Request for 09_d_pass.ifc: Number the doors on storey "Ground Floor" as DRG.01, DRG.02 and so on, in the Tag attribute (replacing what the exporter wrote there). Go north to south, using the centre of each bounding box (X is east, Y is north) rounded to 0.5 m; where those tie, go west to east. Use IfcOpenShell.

First a look at what the model holds.

```python
import ifcopenshell
import ifcopenshell.util.element
import ifcopenshell.util.placement

model = ifcopenshell.open("09_d_pass.ifc")
print(model.schema)
storey = next(s for s in model.by_type("IfcBuildingStorey") if s.Name == "Ground Floor")
doors = [e for e in ifcopenshell.util.element.get_decomposition(storey) if e.is_a("IfcDoor")]
for e in sorted(doors, key=lambda e: e.id()):
    origin = ifcopenshell.util.placement.get_local_placement(e.ObjectPlacement)[:3, 3]
    print(e.id(), e.Tag, e.Name, origin.round(2) + 0.0, sep=" | ")
```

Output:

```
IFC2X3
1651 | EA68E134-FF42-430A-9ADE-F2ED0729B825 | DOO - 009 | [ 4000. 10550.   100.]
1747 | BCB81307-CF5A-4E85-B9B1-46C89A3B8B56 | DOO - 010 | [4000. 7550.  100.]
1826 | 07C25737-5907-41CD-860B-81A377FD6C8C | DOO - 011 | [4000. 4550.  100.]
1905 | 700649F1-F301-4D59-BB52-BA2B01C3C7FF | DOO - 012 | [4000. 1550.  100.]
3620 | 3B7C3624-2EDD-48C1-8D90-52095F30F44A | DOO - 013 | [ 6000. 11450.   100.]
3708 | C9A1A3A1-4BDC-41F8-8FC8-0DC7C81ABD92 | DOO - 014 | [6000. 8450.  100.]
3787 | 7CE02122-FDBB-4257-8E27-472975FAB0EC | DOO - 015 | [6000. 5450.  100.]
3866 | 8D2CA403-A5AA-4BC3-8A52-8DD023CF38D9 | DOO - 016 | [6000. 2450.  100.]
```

```python
import ifcopenshell
import ifcopenshell.geom
import ifcopenshell.util.element
import ifcopenshell.util.shape

model = ifcopenshell.open("09_d_pass.ifc")
settings = ifcopenshell.geom.settings()
settings.set("use-world-coords", True)


def centre(element):
    shape = ifcopenshell.geom.create_shape(settings, element)
    return ifcopenshell.util.shape.get_bbox_centroid(shape.geometry)


storey = next(s for s in model.by_type("IfcBuildingStorey") if s.Name == "Ground Floor")
doors = [e for e in ifcopenshell.util.element.get_decomposition(storey) if e.is_a("IfcDoor")]

# Insertion points can sit at a corner or the storey origin, so sort by the geometry (in metres).
centres = {e: centre(e) for e in doors}
doors.sort(key=lambda e: (-round(centres[e][1] / 0.5), centres[e][0]))

for i, e in enumerate(doors, start=1):
    number = f"DRG.{i:02d}"
    e.Tag = number
    print(e.id(), number)

model.write("09_d_pass_updated.ifc")
```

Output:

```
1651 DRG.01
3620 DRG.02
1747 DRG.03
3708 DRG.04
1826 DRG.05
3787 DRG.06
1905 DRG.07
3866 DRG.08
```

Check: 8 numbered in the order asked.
